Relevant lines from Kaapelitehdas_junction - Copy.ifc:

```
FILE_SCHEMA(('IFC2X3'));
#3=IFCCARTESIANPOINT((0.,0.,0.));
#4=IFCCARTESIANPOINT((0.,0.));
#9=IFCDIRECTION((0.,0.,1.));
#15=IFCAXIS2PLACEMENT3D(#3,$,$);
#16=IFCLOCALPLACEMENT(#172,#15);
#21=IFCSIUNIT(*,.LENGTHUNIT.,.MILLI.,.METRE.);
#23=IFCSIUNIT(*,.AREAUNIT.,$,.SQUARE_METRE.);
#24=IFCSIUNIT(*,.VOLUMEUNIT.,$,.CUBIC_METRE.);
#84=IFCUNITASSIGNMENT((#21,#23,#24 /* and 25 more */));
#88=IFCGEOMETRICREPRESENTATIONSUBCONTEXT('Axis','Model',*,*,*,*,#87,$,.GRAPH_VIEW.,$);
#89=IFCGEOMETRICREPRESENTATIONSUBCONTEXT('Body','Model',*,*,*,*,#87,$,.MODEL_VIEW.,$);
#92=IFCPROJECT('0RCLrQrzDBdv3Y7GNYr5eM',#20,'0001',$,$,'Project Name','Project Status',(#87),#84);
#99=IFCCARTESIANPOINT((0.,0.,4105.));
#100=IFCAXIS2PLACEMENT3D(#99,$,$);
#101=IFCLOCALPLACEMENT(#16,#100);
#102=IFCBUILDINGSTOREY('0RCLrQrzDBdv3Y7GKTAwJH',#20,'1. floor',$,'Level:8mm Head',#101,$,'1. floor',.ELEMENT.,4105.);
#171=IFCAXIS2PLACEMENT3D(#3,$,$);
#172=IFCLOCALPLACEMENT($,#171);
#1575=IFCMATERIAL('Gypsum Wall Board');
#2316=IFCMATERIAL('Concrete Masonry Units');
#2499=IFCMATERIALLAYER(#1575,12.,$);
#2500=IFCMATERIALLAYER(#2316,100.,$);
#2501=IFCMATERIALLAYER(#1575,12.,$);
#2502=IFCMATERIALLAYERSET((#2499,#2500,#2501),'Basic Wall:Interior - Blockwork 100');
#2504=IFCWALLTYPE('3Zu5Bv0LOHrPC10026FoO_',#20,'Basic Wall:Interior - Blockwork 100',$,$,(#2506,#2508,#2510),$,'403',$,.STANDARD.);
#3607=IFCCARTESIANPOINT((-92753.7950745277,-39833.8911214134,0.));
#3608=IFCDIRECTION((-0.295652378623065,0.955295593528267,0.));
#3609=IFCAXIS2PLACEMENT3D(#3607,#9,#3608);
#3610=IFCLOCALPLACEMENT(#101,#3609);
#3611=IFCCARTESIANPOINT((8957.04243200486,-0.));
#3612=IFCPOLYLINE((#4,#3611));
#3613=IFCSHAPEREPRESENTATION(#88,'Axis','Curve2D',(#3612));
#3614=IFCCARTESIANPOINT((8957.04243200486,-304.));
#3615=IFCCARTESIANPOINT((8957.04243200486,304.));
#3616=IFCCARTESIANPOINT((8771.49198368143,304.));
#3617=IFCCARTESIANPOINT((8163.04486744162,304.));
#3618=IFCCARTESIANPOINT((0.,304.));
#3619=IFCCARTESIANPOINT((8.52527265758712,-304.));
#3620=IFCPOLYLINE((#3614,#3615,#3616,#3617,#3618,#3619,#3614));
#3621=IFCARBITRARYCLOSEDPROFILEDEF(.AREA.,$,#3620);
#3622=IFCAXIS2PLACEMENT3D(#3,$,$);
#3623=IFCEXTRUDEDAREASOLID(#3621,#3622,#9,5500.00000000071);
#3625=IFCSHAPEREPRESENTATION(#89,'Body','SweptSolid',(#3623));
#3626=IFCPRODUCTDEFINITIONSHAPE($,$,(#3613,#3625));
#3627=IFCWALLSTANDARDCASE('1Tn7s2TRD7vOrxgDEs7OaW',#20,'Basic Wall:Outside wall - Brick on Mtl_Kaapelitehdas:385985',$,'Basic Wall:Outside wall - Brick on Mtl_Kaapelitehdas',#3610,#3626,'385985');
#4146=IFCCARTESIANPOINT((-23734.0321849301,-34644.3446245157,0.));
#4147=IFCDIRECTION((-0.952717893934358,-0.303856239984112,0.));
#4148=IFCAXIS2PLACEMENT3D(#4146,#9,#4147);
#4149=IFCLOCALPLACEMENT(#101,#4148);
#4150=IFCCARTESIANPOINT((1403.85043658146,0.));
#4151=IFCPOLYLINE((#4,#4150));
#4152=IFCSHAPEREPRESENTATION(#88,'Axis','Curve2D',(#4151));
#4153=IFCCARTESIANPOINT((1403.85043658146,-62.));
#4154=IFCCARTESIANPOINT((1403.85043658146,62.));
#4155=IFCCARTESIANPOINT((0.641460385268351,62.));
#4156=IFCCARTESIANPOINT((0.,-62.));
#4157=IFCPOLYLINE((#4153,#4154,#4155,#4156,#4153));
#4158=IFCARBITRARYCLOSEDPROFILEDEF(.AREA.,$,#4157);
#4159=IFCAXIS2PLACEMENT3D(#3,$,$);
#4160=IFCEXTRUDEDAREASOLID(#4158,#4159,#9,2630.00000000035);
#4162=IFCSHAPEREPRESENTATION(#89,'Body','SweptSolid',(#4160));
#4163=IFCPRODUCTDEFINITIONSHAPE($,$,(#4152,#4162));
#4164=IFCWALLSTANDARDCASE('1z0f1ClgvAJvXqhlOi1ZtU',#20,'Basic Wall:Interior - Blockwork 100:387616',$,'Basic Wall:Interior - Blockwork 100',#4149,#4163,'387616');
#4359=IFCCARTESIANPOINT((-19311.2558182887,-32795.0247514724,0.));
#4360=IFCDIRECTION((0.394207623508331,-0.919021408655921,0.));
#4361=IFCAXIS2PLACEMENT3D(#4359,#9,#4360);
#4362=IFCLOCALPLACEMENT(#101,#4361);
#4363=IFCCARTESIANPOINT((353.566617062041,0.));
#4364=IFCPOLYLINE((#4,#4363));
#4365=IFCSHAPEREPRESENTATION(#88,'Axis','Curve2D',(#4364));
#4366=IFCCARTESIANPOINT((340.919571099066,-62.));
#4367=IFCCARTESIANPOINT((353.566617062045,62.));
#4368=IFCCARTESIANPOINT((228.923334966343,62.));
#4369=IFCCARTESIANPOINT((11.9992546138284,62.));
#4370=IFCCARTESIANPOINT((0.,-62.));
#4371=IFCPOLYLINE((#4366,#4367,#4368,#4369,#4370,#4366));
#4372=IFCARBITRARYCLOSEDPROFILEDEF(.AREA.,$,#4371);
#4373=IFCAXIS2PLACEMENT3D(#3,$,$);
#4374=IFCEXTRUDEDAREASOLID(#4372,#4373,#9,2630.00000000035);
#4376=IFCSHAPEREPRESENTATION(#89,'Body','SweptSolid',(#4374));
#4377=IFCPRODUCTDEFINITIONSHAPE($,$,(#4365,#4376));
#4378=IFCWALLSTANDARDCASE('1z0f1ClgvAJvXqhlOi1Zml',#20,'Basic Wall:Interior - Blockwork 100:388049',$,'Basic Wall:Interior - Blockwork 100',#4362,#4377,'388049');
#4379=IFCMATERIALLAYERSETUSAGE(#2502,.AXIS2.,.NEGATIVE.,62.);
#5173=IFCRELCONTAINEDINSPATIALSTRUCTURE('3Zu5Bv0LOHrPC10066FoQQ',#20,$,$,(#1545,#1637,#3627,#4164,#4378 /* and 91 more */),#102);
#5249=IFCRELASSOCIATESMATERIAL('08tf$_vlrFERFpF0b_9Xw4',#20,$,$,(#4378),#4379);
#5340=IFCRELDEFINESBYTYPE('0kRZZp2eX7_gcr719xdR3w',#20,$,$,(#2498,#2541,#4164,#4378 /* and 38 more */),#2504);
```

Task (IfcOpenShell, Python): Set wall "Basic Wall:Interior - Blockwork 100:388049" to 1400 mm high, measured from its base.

```python
import ifcopenshell
import ifcopenshell.geom
import ifcopenshell.util.representation
import ifcopenshell.util.shape
import ifcopenshell.util.unit

model = ifcopenshell.open("Kaapelitehdas_junction - Copy.ifc")
unit_scale = ifcopenshell.util.unit.calculate_unit_scale(model)
settings = ifcopenshell.geom.settings()


def volume(element):
    """Net volume in cubic metres, openings subtracted."""
    shape = ifcopenshell.geom.create_shape(settings, element)
    return ifcopenshell.util.shape.get_volume(shape.geometry)


wall = model.by_id(4378)
before = volume(wall)

body = ifcopenshell.util.representation.get_representation(wall, "Model", "Body")
solid = body.Items[0]
old_height = solid.Depth
solid.Depth = 1.4 / unit_scale
after = volume(wall)

print(f"height {old_height:g} -> {solid.Depth:g}, volume {before:.3f} -> {after:.3f} m3")

model.write("Kaapelitehdas_junction - Copy-out.ifc")
```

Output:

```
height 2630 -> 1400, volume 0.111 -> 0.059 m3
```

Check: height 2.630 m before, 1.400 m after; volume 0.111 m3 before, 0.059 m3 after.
